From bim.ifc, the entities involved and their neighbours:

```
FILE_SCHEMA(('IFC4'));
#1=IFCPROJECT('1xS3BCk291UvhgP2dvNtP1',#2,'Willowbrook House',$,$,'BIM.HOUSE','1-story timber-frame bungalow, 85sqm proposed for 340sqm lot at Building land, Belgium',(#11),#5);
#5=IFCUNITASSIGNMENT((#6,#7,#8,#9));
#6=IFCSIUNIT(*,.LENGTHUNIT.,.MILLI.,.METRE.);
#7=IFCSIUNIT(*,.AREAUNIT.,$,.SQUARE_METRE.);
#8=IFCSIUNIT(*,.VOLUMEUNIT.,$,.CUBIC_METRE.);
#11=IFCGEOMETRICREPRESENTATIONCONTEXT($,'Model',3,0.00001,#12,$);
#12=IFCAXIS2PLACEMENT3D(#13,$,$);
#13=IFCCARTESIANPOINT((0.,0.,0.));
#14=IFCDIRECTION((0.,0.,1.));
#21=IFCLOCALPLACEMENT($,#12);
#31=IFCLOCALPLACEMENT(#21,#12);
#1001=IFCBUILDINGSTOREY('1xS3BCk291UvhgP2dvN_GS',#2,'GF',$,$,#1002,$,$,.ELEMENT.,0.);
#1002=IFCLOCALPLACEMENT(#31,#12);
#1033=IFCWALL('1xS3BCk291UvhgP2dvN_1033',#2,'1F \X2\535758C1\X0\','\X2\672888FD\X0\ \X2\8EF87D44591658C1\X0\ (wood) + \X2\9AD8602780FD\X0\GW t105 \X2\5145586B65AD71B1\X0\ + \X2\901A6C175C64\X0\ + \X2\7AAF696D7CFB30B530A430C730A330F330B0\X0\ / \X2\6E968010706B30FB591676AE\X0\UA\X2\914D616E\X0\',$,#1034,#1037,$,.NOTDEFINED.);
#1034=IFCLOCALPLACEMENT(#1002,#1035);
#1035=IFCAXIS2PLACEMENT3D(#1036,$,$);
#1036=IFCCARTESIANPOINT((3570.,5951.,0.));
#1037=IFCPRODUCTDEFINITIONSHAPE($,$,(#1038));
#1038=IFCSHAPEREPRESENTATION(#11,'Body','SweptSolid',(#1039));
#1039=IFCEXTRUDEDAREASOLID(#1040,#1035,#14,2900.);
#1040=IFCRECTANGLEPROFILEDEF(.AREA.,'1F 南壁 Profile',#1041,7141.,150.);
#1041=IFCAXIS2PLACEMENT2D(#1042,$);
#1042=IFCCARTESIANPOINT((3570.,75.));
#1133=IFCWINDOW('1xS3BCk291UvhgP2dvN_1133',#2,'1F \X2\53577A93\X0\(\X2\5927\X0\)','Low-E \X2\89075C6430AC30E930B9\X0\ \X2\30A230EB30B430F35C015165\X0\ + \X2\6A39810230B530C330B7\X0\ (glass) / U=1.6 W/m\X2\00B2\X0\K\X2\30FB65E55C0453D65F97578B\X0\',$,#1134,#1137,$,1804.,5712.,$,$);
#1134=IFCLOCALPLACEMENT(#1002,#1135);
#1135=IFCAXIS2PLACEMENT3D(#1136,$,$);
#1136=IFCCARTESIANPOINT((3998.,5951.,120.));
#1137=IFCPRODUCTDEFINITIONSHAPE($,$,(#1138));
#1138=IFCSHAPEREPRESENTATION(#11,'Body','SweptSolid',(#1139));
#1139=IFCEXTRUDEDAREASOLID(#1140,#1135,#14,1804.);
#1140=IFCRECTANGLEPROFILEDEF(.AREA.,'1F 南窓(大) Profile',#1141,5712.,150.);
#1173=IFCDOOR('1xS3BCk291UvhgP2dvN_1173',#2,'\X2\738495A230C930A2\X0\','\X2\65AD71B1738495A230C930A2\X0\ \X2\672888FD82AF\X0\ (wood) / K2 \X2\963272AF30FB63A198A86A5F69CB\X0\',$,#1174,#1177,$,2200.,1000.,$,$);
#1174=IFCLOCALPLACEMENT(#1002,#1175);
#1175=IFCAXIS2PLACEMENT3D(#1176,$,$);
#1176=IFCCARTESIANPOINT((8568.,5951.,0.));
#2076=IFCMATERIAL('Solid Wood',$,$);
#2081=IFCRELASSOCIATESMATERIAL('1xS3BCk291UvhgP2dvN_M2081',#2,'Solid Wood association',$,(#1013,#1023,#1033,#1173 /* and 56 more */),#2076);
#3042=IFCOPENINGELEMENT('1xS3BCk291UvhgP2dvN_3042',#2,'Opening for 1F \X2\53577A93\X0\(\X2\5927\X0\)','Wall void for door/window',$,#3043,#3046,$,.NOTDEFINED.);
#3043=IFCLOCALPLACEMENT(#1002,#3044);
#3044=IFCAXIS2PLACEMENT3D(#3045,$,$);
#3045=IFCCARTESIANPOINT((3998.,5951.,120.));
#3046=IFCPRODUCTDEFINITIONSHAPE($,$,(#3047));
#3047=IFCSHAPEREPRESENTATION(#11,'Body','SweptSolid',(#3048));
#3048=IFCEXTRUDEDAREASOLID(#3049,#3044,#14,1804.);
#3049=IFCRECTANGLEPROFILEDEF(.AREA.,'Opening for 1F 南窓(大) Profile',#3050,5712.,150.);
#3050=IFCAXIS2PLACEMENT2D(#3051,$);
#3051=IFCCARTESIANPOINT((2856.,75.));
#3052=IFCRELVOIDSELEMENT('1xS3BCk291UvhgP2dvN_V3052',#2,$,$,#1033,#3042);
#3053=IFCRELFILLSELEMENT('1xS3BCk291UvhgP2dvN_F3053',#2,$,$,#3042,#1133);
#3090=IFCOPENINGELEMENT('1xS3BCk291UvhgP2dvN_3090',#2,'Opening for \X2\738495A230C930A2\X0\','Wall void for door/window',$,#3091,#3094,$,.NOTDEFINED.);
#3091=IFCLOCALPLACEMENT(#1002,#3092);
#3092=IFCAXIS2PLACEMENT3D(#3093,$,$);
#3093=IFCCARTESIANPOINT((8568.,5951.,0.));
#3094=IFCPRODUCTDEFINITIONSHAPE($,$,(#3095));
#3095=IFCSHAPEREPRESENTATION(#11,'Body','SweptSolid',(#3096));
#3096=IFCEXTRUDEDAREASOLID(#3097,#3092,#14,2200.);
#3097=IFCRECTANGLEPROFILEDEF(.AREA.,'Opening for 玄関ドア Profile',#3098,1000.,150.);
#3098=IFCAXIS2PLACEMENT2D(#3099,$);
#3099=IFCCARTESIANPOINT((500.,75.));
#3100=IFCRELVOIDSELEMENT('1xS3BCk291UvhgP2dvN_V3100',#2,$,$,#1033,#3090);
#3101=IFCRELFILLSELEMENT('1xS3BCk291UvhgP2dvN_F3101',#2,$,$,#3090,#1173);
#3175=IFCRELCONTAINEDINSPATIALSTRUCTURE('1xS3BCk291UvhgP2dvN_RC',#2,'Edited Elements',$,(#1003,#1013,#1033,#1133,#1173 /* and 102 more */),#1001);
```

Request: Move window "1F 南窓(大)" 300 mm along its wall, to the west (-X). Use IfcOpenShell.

```python
import ifcopenshell
import ifcopenshell.api.geometry
import ifcopenshell.util.placement

model = ifcopenshell.open("bim.ifc")

window = model.by_id(1133)
opening = window.FillsVoids[0].RelatingOpeningElement
wall = opening.VoidsElements[0].RelatingBuildingElement

wall_matrix = ifcopenshell.util.placement.get_local_placement(wall.ObjectPlacement)
shift = wall_matrix[:3, 0] * -300.0
before = ifcopenshell.util.placement.get_local_placement(window.ObjectPlacement)[:3, 3].copy()

# The window is not placed relative to its opening, so move both.
for product in (opening, window):
    matrix = ifcopenshell.util.placement.get_local_placement(product.ObjectPlacement)
    matrix[:3, 3] += shift
    ifcopenshell.api.geometry.edit_object_placement(model, product=product, matrix=matrix, is_si=False)

after = ifcopenshell.util.placement.get_local_placement(window.ObjectPlacement)[:3, 3]
print("window moved by", (after - before).round(3) + 0.0)

model.write("bim_edited.ifc")
```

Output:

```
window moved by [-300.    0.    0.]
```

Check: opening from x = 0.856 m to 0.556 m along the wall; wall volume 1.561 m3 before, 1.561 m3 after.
